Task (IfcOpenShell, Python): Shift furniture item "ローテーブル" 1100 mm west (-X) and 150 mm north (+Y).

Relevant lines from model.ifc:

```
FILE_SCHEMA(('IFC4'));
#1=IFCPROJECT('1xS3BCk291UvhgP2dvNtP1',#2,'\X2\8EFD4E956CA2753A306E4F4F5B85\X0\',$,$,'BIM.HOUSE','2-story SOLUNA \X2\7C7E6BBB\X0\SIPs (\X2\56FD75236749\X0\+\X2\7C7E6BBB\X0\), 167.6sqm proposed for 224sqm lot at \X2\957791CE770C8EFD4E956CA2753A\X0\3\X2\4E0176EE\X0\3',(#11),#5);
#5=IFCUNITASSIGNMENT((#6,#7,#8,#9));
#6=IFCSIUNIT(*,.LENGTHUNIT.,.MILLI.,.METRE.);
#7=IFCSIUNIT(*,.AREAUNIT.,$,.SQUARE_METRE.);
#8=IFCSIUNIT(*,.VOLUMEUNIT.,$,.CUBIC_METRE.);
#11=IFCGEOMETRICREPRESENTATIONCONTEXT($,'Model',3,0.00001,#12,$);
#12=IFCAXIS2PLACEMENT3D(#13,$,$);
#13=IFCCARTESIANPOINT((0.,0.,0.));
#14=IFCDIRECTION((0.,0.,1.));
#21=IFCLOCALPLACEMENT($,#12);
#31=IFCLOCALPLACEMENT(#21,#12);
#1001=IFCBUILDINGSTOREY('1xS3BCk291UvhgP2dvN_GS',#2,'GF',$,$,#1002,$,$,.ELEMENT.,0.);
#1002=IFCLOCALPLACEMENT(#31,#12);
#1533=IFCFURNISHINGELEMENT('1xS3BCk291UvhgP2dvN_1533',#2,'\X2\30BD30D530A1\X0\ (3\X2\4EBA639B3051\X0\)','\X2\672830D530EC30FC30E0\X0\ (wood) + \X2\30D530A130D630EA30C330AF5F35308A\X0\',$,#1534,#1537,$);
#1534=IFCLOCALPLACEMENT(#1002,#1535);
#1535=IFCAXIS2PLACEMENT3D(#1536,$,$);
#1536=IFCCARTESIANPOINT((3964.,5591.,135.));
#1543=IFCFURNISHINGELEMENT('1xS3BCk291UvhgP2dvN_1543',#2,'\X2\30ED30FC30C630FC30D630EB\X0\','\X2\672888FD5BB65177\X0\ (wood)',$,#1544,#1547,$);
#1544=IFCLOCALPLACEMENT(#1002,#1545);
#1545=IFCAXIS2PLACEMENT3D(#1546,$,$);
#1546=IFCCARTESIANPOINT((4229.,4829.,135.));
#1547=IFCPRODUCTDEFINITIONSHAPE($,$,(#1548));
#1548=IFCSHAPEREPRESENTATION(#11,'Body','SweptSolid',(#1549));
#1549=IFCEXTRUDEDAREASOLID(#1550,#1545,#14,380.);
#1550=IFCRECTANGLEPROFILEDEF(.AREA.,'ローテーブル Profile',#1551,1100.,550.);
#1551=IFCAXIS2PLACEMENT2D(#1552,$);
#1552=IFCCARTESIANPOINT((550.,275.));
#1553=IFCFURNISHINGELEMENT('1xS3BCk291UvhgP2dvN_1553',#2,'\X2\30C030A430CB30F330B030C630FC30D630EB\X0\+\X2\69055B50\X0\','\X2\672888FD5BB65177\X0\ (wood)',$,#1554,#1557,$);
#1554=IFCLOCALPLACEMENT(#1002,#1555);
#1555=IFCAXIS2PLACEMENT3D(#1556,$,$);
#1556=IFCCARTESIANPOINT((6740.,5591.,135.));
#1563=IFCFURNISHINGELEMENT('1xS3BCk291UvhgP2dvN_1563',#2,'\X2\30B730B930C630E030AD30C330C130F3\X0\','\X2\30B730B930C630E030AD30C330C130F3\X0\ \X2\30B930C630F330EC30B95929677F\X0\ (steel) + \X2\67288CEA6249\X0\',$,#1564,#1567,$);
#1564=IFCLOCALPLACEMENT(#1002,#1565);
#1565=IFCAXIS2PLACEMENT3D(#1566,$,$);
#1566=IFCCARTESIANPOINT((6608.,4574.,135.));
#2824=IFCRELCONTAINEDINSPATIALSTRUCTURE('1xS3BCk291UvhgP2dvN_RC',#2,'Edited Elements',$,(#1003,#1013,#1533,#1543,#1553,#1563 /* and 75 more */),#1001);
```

```python
import ifcopenshell
import ifcopenshell.api.geometry
import ifcopenshell.util.placement
import ifcopenshell.util.unit

model = ifcopenshell.open("model.ifc")
unit_scale = ifcopenshell.util.unit.calculate_unit_scale(model)

item = model.by_id(1543)
matrix = ifcopenshell.util.placement.get_local_placement(item.ObjectPlacement)
matrix[0, 3] -= 1.1 / unit_scale
matrix[1, 3] += 0.15 / unit_scale
ifcopenshell.api.geometry.edit_object_placement(model, product=item, matrix=matrix, is_si=False)

print(ifcopenshell.util.placement.get_local_placement(item.ObjectPlacement).round(3) + 0.0)

model.write("model_v2.ifc")
```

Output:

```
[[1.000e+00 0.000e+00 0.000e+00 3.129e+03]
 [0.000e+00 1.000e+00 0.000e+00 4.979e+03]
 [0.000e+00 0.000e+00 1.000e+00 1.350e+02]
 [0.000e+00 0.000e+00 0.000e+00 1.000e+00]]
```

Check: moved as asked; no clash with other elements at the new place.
